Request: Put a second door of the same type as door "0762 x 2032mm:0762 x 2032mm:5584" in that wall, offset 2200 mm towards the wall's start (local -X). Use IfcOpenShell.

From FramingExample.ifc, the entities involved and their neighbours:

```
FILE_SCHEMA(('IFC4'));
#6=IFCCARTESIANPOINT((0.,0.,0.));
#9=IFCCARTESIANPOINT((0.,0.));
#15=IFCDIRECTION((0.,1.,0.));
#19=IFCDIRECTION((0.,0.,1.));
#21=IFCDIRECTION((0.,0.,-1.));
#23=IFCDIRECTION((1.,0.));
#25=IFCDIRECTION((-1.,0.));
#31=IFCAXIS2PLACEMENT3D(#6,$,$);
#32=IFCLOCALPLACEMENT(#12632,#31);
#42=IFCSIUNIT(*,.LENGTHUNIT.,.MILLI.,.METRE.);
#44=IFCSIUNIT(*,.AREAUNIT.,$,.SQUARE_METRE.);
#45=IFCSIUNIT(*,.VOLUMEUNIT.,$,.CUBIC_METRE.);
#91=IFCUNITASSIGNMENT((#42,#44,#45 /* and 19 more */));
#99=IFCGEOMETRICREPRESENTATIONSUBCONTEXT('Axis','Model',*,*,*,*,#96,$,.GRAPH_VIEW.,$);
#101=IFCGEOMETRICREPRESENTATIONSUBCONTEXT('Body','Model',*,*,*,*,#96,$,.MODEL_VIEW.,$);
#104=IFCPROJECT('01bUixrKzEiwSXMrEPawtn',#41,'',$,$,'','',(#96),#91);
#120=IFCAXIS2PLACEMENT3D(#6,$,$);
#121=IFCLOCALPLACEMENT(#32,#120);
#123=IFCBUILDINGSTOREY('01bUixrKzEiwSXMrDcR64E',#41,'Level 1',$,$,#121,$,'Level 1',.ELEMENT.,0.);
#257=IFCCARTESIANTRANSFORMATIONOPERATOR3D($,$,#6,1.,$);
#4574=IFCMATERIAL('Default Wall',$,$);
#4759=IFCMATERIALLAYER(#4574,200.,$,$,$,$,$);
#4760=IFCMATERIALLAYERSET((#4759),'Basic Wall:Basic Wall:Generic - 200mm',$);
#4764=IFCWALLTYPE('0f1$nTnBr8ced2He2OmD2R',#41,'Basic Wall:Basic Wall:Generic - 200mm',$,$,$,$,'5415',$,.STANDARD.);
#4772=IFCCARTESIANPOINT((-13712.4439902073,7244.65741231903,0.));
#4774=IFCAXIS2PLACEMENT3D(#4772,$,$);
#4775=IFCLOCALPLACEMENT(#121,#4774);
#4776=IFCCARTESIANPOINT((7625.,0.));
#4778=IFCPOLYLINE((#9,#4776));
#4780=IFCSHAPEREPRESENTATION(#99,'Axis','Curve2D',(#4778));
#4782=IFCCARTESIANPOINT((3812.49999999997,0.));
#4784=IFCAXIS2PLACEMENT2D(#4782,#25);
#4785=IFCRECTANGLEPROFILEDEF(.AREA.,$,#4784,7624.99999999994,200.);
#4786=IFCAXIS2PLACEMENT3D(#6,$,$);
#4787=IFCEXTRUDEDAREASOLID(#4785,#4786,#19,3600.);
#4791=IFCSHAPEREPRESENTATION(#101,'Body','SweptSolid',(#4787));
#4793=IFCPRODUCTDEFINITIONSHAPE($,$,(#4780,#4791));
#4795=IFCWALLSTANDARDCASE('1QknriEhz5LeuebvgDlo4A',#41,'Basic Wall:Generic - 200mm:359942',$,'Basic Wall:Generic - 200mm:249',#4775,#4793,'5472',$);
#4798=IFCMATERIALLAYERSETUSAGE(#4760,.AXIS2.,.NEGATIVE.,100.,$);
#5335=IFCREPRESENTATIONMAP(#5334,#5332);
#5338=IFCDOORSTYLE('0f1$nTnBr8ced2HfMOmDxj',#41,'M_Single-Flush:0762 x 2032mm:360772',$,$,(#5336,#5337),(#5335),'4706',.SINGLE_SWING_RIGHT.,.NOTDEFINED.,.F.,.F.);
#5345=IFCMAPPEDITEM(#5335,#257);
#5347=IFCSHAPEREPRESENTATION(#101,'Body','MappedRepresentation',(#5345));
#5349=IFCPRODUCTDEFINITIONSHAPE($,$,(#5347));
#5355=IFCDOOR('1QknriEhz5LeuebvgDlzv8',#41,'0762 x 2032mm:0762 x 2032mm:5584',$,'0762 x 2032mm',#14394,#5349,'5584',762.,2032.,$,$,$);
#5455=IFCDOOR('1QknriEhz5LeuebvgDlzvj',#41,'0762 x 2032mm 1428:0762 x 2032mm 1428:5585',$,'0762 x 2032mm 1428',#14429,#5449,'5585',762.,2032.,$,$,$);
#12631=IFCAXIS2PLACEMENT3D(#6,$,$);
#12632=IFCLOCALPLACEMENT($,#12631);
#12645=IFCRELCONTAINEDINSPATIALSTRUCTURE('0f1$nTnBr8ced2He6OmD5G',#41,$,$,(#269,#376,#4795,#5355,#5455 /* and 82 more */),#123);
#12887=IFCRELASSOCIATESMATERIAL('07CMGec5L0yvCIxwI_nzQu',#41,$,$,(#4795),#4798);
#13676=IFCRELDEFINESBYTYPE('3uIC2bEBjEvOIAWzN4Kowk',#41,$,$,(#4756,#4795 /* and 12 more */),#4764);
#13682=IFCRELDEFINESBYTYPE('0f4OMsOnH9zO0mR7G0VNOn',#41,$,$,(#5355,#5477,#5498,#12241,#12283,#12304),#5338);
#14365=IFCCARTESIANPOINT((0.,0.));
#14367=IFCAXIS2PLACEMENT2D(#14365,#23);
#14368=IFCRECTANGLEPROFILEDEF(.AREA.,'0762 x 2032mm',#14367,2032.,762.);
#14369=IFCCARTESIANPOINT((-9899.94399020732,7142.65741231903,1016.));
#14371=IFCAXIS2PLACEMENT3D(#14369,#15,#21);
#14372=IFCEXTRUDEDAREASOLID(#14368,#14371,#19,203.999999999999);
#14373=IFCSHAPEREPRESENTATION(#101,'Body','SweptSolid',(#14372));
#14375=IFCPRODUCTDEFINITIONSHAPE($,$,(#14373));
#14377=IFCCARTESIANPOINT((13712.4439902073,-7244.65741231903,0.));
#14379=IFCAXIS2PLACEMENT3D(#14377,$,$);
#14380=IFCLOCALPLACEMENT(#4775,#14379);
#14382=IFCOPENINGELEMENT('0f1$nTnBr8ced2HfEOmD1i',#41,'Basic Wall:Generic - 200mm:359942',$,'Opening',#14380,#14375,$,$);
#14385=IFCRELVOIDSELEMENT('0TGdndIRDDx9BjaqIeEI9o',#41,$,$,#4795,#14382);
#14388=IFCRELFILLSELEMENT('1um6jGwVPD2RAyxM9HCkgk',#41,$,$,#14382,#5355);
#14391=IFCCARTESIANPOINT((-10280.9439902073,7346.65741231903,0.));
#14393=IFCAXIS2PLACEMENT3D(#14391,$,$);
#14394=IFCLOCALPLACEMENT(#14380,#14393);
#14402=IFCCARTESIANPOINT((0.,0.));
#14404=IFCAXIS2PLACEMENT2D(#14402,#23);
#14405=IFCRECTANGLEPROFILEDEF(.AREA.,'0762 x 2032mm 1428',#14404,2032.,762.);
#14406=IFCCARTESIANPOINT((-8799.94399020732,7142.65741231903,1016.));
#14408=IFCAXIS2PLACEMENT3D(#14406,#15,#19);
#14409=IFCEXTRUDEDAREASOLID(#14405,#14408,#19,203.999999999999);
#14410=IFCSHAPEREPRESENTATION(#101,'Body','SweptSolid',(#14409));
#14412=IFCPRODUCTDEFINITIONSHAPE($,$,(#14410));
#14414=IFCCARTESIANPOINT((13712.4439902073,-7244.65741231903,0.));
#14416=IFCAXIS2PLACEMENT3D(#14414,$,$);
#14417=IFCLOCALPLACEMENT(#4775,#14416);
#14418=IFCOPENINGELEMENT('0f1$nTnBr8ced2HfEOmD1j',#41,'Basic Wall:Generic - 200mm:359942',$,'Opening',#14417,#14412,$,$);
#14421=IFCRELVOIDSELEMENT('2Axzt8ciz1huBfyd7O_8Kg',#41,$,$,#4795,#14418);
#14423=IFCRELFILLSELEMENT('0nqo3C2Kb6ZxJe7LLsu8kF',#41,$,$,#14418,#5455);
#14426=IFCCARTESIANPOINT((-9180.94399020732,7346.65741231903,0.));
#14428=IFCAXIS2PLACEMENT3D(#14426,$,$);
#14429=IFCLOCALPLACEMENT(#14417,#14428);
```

```python
import ifcopenshell
import ifcopenshell.api.feature
import ifcopenshell.api.geometry
import ifcopenshell.api.root
import ifcopenshell.geom
import ifcopenshell.util.element
import ifcopenshell.util.placement
import ifcopenshell.util.shape

model = ifcopenshell.open("FramingExample.ifc")
settings = ifcopenshell.geom.settings()


def volume(element):
    """Net volume in cubic metres, openings subtracted."""
    shape = ifcopenshell.geom.create_shape(settings, element)
    return ifcopenshell.util.shape.get_volume(shape.geometry)


def reuse_history(source, copy):
    """copy_class also copies each property set's owner history, people and application; keep the originals."""
    for rel in copy.IsDefinedBy:
        if rel.is_a("IfcRelDefinesByProperties") and (history := rel.RelatingPropertyDefinition.OwnerHistory):
            rel.RelatingPropertyDefinition.OwnerHistory = source.OwnerHistory
            ifcopenshell.util.element.remove_deep2(model, history)


door = model.by_id(5355)
opening = door.FillsVoids[0].RelatingOpeningElement
wall = opening.VoidsElements[0].RelatingBuildingElement
before = volume(wall)
shift = ifcopenshell.util.placement.get_local_placement(wall.ObjectPlacement)[:3, 0] * -2200.0

# copy_class copies the void relationship, type, container and properties, but no geometry.
new_opening = ifcopenshell.api.root.copy_class(model, product=opening)
new_opening.Representation = ifcopenshell.util.element.copy_deep(
    model, opening.Representation, exclude=["IfcGeometricRepresentationContext", "IfcRepresentationMap"]
)
new_opening.Name = "Basic Wall:Generic - 200mm"
new_door = ifcopenshell.api.root.copy_class(model, product=door)
new_door.Representation = ifcopenshell.util.element.copy_deep(
    model, door.Representation, exclude=["IfcGeometricRepresentationContext", "IfcRepresentationMap"]
)
new_door.Name = "0762 x 2032mm:0762 x 2032mm"
new_door.Tag = None
reuse_history(door, new_door)
ifcopenshell.api.feature.add_filling(model, opening=new_opening, element=new_door)

for old, new in ((opening, new_opening), (door, new_door)):
    matrix = ifcopenshell.util.placement.get_local_placement(old.ObjectPlacement)
    matrix[:3, 3] += shift
    ifcopenshell.api.geometry.edit_object_placement(model, product=new, matrix=matrix, is_si=False)

after = volume(wall)

print(f"wall volume {before:.3f} -> {after:.3f} m3")

model.write("FramingExample_rev.ifc")
```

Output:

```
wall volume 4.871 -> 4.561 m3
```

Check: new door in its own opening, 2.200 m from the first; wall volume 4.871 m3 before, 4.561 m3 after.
